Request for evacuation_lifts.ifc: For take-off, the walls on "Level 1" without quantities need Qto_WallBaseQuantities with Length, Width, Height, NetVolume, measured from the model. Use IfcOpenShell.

First a look at what the model holds.

```python
import ifcopenshell
import ifcopenshell.util.element
import ifcopenshell.util.unit

model = ifcopenshell.open("evacuation_lifts.ifc")
print(model.schema)
for unit_type in ("LENGTHUNIT", "AREAUNIT", "VOLUMEUNIT"):
    print(unit_type, ifcopenshell.util.unit.calculate_unit_scale(model, unit_type))
storey = next(s for s in model.by_type("IfcBuildingStorey") if s.Name == "Level 1")
walls = [e for e in ifcopenshell.util.element.get_decomposition(storey) if e.is_a("IfcWall")]
for e in sorted(walls, key=lambda e: e.id()):
    print(e.id(), e.is_a(), e.Name, list(ifcopenshell.util.element.get_psets(e, qtos_only=True)), sep=" | ")
```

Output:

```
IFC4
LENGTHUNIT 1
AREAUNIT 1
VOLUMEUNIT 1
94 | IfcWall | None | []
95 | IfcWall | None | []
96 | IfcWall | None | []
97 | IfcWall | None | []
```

```python
import ifcopenshell
import ifcopenshell.api.pset
import ifcopenshell.geom
import ifcopenshell.util.element
import ifcopenshell.util.shape
import ifcopenshell.util.unit

model = ifcopenshell.open("evacuation_lifts.ifc")
unit_scale = ifcopenshell.util.unit.calculate_unit_scale(model)
volume_scale = ifcopenshell.util.unit.calculate_unit_scale(model, "VOLUMEUNIT")
settings = ifcopenshell.geom.settings()

storey = next(s for s in model.by_type("IfcBuildingStorey") if s.Name == "Level 1")
walls = [e for e in ifcopenshell.util.element.get_decomposition(storey) if e.is_a("IfcWall")]

for e in sorted(walls, key=lambda e: e.id()):
    if ifcopenshell.util.element.get_psets(e, qtos_only=True, should_inherit=False):
        continue
    # Geometry comes back in metres, in the element's own axes.
    shape = ifcopenshell.geom.create_shape(settings, e)
    values = {
        "Length": ifcopenshell.util.shape.get_x(shape.geometry) / unit_scale,
        "Width": ifcopenshell.util.shape.get_y(shape.geometry) / unit_scale,
        "Height": ifcopenshell.util.shape.get_z(shape.geometry) / unit_scale,
        "NetVolume": ifcopenshell.util.shape.get_volume(shape.geometry) / volume_scale,
    }
    qto = ifcopenshell.api.pset.add_qto(model, product=e, name="Qto_WallBaseQuantities")
    ifcopenshell.api.pset.edit_qto(model, qto=qto, properties=values)
    print(e.id(), {k: round(v, 3) for k, v in values.items()})

model.write("evacuation_lifts_v2.ifc")
```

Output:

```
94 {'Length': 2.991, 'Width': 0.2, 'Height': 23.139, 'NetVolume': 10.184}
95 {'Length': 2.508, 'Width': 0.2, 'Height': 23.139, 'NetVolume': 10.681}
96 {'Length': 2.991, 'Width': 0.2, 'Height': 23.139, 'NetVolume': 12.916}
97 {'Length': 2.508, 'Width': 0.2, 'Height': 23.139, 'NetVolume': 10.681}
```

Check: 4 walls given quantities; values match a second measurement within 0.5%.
